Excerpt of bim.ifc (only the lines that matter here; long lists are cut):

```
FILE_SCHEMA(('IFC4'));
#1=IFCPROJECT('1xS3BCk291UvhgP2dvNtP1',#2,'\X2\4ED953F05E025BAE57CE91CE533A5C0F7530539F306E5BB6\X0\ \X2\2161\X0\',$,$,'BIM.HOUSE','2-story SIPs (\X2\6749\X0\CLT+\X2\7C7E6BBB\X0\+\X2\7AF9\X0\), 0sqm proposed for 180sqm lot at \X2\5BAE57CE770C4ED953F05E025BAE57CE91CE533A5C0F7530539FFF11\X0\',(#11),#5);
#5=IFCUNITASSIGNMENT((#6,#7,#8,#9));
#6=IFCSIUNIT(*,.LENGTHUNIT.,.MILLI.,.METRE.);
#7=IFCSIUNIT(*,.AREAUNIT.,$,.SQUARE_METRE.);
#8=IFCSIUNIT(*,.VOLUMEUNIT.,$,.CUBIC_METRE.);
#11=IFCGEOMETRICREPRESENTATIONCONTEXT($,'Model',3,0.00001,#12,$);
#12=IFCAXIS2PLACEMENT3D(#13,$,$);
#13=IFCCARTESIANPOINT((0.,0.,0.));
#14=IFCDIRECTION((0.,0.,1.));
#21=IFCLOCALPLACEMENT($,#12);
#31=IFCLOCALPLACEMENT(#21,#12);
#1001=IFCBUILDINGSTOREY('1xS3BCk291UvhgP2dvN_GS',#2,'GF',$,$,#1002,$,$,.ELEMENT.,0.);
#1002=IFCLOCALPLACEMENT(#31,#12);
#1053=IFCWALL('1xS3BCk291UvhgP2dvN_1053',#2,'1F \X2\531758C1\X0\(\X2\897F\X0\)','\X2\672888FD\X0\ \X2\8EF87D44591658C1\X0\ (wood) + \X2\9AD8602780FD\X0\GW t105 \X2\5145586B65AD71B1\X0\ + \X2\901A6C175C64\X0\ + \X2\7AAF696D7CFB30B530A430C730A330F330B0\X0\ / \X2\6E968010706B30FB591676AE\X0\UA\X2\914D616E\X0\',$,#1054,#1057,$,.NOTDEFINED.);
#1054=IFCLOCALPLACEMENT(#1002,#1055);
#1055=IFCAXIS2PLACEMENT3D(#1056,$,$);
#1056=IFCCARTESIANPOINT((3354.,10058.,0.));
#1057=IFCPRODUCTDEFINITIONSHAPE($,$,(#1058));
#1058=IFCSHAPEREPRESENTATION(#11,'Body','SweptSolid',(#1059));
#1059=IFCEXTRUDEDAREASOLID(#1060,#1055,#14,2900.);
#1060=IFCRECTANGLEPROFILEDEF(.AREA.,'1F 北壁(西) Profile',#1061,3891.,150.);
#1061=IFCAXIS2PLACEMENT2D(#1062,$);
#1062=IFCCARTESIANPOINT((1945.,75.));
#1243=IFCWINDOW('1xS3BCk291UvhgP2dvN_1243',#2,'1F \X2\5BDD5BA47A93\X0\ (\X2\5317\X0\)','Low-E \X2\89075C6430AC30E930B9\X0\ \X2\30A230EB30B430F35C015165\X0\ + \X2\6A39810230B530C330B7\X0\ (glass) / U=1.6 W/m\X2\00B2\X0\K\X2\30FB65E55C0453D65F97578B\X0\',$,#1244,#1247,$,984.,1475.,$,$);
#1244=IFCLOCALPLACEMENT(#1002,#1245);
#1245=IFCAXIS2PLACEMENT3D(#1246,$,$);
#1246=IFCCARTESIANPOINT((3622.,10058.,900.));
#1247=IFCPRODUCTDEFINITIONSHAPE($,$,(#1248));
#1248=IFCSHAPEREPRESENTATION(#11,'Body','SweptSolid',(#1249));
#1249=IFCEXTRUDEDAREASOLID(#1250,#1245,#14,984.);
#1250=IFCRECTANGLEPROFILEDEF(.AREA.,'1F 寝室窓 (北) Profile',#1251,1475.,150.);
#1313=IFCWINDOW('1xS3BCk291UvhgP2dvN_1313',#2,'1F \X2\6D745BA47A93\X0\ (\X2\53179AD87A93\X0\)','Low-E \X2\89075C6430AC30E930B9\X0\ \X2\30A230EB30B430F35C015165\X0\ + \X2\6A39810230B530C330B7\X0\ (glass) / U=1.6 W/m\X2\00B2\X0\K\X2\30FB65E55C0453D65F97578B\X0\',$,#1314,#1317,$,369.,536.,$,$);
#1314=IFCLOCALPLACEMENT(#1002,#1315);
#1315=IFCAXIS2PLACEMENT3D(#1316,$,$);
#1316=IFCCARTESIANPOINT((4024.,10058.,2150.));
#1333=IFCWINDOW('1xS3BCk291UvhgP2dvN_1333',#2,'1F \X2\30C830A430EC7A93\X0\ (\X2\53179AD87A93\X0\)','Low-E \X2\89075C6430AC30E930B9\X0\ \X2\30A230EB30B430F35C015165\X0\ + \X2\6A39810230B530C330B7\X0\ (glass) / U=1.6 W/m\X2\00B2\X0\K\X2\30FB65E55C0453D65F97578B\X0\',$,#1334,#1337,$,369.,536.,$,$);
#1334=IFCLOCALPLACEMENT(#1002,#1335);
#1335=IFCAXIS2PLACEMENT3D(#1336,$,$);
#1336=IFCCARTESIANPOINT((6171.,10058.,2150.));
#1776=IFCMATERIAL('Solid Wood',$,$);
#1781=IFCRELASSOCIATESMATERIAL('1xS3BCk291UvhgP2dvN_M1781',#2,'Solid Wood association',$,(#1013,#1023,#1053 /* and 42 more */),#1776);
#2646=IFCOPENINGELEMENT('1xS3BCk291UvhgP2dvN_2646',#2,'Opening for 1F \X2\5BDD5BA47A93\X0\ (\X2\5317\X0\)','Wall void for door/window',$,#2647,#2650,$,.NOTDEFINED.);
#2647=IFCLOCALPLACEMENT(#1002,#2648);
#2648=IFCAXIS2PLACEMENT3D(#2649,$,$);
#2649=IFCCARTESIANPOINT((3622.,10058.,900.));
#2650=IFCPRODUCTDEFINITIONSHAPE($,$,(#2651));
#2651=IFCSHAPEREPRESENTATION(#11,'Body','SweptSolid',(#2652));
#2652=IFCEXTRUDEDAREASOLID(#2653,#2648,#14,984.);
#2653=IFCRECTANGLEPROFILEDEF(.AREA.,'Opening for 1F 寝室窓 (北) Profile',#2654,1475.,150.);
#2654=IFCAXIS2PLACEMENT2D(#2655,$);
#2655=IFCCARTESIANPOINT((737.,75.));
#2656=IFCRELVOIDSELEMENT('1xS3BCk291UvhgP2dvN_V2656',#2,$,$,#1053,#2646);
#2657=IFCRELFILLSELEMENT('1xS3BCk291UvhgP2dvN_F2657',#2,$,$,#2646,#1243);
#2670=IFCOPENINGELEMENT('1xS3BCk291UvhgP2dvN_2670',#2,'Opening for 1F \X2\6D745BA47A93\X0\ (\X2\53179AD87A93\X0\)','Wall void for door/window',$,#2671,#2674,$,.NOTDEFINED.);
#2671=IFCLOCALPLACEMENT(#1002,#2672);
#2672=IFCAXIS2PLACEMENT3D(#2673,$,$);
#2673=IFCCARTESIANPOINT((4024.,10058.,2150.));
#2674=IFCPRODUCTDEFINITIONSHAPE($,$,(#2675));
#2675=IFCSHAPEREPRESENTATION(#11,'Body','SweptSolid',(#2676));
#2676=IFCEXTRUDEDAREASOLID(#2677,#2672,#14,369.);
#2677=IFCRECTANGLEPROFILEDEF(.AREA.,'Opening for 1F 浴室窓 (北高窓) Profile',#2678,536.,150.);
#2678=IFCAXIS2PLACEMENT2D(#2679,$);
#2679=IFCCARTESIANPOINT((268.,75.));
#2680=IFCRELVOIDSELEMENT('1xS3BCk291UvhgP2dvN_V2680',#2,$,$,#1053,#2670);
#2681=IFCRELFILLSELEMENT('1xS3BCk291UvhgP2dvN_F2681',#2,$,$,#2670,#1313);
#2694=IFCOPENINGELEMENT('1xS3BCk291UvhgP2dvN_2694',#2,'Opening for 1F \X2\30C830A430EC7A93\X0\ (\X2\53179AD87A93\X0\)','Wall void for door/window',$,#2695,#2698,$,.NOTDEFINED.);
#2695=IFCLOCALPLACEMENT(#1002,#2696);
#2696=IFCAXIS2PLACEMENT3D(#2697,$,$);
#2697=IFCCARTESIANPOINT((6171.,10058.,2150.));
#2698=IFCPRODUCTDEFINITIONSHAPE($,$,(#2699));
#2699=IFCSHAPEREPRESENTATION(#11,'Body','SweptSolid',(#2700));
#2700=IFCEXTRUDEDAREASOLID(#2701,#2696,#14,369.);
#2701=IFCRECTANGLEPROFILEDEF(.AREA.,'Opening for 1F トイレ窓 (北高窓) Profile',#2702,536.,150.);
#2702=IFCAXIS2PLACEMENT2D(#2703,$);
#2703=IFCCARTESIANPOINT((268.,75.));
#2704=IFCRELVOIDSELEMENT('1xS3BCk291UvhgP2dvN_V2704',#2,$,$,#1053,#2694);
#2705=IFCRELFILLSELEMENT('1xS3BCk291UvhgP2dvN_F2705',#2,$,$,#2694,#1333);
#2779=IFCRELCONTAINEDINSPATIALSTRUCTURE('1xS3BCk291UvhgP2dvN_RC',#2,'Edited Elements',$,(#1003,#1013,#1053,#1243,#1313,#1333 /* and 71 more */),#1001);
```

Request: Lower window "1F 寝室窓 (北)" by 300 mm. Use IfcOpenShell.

```python
import numpy as np
import ifcopenshell
import ifcopenshell.api.geometry
import ifcopenshell.util.placement
import ifcopenshell.util.unit

model = ifcopenshell.open("bim.ifc")
unit_scale = ifcopenshell.util.unit.calculate_unit_scale(model)

window = model.by_guid("1xS3BCk291UvhgP2dvN_1243")
opening = window.FillsVoids[0].RelatingOpeningElement
dz = -0.3 / unit_scale

shift = np.array([0.0, 0.0, dz])
# The window is not placed relative to its opening, so move both.
for product in (opening, window):
    matrix = ifcopenshell.util.placement.get_local_placement(product.ObjectPlacement)
    matrix[:3, 3] += shift
    ifcopenshell.api.geometry.edit_object_placement(model, product=product, matrix=matrix, is_si=False)

print(f"moved by {dz * unit_scale:+.3f} m")

model.write("bim_rev.ifc")
```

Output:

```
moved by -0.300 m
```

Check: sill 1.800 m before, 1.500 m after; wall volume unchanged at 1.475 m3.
